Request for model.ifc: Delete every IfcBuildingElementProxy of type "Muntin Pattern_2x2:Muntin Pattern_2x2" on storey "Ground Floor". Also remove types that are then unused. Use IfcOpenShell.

First a look at what the model holds.

```python
import ifcopenshell
import ifcopenshell.util.element

model = ifcopenshell.open("model.ifc")
print(model.schema)
storey = next(s for s in model.by_type("IfcBuildingStorey") if s.Name == "Ground Floor")
proxies = [e for e in ifcopenshell.util.element.get_decomposition(storey) if e.is_a("IfcBuildingElementProxy")]
seen = {}
for e in proxies:
    element_type = ifcopenshell.util.element.get_type(e)
    name = element_type.Name if element_type not in (None, e) else None
    seen[name] = seen.get(name, 0) + 1
for name, count in sorted(seen.items(), key=str):
    print(count, "x", name)
```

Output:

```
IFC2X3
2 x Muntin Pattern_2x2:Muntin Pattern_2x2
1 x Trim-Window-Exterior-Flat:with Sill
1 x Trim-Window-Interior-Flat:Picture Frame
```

```python
import ifcopenshell
import ifcopenshell.api.root
import ifcopenshell.util.element

model = ifcopenshell.open("model.ifc")

storey = next(s for s in model.by_type("IfcBuildingStorey") if s.Name == "Ground Floor")
proxies = [e for e in ifcopenshell.util.element.get_decomposition(storey) if e.is_a("IfcBuildingElementProxy")]
targets = [e for e in proxies if (t := ifcopenshell.util.element.get_type(e)) not in (None, e) and t.Name == "Muntin Pattern_2x2:Muntin Pattern_2x2"]
types = {ifcopenshell.util.element.get_type(e) for e in targets} - {None, *targets}

for e in targets:
    ifcopenshell.api.root.remove_product(model, product=e)
print(len(targets), "removed")

unused = [t for t in types if not ifcopenshell.util.element.get_types(t)]
for t in unused:
    ifcopenshell.api.root.remove_product(model, product=t)
print(len(unused), "unused types removed")

model.write("model_v2.ifc")
```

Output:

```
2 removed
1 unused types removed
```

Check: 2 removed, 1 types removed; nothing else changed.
